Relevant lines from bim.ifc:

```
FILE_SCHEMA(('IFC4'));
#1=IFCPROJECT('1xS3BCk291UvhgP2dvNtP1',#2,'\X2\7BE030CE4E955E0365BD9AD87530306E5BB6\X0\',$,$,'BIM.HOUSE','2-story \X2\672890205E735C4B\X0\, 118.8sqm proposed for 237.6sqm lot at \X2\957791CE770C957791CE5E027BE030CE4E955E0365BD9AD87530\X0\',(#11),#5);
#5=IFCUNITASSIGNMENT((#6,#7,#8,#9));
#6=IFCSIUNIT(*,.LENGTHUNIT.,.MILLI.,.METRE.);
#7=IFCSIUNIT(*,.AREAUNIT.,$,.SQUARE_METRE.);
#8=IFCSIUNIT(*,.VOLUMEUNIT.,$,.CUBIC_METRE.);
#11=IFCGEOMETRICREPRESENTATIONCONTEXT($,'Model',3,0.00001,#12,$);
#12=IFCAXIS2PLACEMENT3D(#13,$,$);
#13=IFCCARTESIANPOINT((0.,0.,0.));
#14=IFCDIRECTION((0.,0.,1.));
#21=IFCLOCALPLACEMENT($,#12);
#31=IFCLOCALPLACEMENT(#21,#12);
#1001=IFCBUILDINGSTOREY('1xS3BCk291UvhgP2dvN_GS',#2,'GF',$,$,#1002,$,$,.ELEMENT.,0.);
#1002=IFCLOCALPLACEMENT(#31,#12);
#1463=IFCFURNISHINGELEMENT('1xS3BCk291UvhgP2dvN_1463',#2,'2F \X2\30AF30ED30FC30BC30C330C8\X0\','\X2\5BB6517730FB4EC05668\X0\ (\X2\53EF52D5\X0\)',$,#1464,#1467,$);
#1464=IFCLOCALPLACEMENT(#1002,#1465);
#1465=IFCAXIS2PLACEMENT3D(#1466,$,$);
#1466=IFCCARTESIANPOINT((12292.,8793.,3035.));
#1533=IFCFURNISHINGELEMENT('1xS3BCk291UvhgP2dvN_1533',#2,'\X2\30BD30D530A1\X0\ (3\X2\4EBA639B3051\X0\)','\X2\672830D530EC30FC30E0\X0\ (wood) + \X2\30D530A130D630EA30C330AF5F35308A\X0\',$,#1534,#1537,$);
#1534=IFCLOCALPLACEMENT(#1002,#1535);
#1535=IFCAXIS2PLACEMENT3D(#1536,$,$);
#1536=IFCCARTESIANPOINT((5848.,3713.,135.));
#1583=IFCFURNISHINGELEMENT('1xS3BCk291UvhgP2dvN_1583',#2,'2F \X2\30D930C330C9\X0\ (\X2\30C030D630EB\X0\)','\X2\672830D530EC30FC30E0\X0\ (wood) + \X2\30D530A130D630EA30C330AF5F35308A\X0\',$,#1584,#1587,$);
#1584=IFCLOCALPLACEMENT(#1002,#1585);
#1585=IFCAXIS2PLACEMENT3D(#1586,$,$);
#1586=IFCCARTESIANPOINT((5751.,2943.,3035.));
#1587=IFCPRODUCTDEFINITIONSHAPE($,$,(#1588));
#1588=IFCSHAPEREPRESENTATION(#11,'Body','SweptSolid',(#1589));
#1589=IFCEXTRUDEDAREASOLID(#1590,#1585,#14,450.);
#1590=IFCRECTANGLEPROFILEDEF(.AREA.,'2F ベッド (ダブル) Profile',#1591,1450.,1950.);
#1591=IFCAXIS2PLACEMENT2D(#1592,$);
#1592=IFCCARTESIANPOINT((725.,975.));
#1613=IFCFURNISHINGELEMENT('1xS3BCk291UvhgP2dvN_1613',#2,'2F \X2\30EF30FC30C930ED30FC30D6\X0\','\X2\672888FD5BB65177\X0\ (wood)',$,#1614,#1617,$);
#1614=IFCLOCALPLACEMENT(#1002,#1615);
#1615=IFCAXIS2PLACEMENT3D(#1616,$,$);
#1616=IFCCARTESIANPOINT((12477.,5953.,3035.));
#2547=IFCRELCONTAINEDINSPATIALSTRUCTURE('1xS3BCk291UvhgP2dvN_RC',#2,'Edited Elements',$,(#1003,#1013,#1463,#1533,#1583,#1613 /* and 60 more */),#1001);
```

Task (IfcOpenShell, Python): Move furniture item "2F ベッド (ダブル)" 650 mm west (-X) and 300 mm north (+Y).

```python
import ifcopenshell
import ifcopenshell.api.geometry
import ifcopenshell.util.placement

model = ifcopenshell.open("bim.ifc")

item = model.by_id(1583)
matrix = ifcopenshell.util.placement.get_local_placement(item.ObjectPlacement)
matrix[0, 3] -= 650.0
matrix[1, 3] += 300.0
ifcopenshell.api.geometry.edit_object_placement(model, product=item, matrix=matrix, is_si=False)

print(ifcopenshell.util.placement.get_local_placement(item.ObjectPlacement).round(3) + 0.0)

model.write("bim_updated.ifc")
```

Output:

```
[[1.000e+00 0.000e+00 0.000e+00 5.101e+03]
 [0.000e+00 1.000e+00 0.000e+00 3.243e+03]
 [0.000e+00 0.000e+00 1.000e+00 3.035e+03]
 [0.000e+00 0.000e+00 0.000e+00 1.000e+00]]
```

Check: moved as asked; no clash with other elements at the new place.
